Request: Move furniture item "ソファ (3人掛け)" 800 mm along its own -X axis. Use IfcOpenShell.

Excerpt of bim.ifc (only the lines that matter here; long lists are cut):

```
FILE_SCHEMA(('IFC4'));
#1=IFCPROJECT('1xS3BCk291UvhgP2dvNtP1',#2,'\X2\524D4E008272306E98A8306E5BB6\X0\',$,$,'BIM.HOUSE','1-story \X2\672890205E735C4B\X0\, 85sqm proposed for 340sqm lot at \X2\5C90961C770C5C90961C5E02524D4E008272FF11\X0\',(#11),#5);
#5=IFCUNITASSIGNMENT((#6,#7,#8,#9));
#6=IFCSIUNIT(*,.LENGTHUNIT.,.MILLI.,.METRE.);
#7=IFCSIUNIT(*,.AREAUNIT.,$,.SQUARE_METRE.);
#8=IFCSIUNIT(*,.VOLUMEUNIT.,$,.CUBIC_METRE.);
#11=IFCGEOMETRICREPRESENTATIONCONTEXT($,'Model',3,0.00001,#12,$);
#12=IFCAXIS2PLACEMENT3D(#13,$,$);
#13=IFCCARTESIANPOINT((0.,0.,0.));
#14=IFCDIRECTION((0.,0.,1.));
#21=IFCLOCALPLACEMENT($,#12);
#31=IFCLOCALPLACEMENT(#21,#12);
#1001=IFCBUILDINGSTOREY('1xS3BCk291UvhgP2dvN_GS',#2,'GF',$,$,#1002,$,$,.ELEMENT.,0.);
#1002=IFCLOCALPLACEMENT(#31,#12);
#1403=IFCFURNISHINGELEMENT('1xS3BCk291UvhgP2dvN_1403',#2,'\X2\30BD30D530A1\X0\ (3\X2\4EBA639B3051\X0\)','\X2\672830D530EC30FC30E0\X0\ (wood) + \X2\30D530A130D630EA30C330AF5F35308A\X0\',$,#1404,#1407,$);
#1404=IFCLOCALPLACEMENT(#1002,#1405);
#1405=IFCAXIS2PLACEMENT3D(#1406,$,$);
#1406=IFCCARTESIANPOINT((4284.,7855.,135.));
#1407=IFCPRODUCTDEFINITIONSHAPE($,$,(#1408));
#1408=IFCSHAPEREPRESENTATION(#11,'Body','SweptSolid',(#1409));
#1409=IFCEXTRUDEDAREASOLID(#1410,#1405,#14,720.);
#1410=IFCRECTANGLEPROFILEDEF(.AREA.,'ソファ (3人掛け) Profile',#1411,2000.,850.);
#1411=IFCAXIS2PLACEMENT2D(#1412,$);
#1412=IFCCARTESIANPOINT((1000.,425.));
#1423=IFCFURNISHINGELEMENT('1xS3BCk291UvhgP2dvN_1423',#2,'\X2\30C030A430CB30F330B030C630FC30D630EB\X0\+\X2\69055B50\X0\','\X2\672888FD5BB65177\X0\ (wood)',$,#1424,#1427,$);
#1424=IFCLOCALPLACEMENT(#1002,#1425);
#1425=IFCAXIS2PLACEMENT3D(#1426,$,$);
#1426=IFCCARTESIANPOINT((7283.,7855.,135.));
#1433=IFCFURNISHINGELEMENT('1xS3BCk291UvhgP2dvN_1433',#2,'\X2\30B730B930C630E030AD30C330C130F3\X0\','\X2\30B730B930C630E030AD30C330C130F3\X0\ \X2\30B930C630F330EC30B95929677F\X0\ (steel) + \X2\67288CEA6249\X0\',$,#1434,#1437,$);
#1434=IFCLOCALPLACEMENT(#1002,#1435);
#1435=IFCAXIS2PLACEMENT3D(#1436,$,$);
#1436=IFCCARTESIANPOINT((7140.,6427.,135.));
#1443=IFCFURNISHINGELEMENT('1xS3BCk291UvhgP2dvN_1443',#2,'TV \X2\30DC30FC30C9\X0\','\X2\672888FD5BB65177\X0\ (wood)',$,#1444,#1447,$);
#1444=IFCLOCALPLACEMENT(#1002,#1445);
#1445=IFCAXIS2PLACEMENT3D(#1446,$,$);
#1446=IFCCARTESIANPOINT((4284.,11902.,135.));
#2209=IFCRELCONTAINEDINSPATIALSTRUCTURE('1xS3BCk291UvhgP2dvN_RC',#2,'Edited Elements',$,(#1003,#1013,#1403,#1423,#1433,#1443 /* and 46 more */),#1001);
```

```python
import ifcopenshell
import ifcopenshell.api.geometry
import ifcopenshell.util.placement

model = ifcopenshell.open("bim.ifc")

item = model.by_guid("1xS3BCk291UvhgP2dvN_1403")
matrix = ifcopenshell.util.placement.get_local_placement(item.ObjectPlacement)
matrix[:3, 3] -= matrix[:3, 0] * 800.0
ifcopenshell.api.geometry.edit_object_placement(model, product=item, matrix=matrix, is_si=False)

print(ifcopenshell.util.placement.get_local_placement(item.ObjectPlacement).round(3) + 0.0)

model.write("bim_updated.ifc")
```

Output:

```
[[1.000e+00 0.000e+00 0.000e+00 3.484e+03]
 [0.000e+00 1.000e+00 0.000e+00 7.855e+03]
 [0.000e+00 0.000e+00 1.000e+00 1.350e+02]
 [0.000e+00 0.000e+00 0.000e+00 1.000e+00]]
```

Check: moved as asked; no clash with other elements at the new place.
